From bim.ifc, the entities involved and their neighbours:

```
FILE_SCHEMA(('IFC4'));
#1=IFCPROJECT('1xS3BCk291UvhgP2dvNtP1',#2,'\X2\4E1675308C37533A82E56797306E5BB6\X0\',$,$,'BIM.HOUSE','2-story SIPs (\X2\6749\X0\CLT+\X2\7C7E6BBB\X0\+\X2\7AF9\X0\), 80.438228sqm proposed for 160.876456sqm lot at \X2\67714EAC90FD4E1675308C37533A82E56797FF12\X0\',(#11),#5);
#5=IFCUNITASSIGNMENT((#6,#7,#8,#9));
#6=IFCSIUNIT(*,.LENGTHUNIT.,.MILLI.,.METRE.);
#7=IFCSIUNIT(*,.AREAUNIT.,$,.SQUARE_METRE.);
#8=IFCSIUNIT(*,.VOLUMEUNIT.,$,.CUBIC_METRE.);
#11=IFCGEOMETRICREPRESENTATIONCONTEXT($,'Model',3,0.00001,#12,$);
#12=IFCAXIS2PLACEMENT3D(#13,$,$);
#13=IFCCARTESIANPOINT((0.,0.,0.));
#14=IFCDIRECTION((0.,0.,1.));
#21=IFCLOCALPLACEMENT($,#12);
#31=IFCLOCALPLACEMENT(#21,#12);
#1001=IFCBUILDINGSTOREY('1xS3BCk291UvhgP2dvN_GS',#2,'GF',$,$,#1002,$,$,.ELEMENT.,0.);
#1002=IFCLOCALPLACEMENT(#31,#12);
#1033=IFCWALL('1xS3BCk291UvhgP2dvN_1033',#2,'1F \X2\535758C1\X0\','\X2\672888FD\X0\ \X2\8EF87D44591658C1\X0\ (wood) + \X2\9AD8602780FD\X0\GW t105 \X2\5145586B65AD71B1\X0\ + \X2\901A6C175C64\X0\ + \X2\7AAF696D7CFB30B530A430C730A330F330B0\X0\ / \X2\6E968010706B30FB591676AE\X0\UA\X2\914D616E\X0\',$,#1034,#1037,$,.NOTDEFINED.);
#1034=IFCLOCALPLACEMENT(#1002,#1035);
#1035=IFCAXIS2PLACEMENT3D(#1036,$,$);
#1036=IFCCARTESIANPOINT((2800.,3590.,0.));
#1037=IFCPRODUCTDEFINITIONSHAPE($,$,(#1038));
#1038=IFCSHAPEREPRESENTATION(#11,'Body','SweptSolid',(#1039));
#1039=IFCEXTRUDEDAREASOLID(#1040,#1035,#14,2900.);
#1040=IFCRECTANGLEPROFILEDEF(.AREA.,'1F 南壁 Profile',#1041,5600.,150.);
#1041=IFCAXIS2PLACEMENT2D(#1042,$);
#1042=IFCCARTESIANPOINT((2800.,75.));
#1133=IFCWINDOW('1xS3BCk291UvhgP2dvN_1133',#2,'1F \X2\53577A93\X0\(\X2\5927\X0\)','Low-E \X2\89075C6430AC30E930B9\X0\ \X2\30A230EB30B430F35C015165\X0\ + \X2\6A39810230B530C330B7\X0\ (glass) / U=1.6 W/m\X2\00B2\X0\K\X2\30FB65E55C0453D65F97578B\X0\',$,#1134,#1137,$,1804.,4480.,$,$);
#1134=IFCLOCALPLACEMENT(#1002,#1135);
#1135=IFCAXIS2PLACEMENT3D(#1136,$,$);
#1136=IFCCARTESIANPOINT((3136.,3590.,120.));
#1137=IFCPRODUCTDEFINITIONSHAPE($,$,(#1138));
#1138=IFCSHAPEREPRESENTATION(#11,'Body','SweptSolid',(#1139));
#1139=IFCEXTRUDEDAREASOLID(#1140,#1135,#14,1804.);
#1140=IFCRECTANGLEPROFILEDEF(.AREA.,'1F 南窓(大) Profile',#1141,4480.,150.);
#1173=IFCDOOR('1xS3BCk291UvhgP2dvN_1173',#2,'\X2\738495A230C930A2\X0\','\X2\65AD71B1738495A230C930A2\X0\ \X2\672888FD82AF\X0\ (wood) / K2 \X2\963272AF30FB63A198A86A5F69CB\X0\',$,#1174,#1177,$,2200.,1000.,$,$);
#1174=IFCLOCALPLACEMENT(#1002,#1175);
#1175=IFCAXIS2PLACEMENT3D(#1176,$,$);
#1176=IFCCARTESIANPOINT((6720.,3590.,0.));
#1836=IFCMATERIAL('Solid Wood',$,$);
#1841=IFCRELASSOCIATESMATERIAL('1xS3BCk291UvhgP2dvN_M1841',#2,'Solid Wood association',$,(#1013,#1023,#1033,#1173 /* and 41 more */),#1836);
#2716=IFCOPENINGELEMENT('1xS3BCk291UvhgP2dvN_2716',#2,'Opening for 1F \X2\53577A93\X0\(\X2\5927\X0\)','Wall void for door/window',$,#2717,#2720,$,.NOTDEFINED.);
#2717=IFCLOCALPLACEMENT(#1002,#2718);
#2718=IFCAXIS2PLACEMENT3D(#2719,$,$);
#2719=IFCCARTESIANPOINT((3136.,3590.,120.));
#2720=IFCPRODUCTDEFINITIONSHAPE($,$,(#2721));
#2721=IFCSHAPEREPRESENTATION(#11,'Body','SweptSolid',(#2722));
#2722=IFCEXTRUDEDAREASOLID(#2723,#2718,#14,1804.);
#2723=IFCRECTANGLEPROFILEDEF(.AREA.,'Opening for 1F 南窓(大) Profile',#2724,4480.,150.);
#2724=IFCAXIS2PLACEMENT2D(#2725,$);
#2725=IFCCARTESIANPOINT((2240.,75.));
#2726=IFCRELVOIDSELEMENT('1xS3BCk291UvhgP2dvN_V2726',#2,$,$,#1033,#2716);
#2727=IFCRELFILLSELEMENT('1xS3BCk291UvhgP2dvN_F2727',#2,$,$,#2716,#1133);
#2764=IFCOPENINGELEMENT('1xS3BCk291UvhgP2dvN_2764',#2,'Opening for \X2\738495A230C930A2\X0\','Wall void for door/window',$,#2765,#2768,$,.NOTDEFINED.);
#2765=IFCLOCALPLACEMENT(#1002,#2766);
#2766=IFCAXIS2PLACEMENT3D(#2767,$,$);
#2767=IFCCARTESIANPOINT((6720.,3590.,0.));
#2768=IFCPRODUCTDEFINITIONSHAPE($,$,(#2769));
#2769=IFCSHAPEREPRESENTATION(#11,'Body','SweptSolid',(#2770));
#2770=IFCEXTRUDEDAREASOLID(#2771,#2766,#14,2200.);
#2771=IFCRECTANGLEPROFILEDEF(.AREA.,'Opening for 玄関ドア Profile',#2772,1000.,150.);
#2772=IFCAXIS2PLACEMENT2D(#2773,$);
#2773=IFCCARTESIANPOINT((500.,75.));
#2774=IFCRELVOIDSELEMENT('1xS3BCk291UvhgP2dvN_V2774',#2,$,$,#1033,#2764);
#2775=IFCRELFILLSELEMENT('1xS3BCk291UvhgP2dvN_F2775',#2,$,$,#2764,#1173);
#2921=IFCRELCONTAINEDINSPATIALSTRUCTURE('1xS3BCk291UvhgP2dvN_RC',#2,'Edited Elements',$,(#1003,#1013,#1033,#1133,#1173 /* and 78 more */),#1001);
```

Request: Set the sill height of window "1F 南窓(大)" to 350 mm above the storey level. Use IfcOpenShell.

```python
import numpy as np
import ifcopenshell
import ifcopenshell.api.geometry
import ifcopenshell.geom
import ifcopenshell.util.element
import ifcopenshell.util.placement
import ifcopenshell.util.shape
import ifcopenshell.util.unit

model = ifcopenshell.open("bim.ifc")
unit_scale = ifcopenshell.util.unit.calculate_unit_scale(model)

window = model.by_guid("1xS3BCk291UvhgP2dvN_1133")
opening = window.FillsVoids[0].RelatingOpeningElement
storey = ifcopenshell.util.element.get_container(window, ifc_class="IfcBuildingStorey")
level = ifcopenshell.util.placement.get_local_placement(storey.ObjectPlacement)[2, 3]

# The opening's origin need not be at the sill, so measure its lowest point.
shape = ifcopenshell.geom.create_shape(ifcopenshell.geom.settings(), opening)
bottom = ifcopenshell.util.shape.get_shape_bottom_elevation(shape, shape.geometry) / unit_scale
dz = level + 350.0 - bottom

shift = np.array([0.0, 0.0, dz])
# The window is not placed relative to its opening, so move both.
for product in (opening, window):
    matrix = ifcopenshell.util.placement.get_local_placement(product.ObjectPlacement)
    matrix[:3, 3] += shift
    ifcopenshell.api.geometry.edit_object_placement(model, product=product, matrix=matrix, is_si=False)

print(f"moved by {dz * unit_scale:+.3f} m")

model.write("bim_edited.ifc")
```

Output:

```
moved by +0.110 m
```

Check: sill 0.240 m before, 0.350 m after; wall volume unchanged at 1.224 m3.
